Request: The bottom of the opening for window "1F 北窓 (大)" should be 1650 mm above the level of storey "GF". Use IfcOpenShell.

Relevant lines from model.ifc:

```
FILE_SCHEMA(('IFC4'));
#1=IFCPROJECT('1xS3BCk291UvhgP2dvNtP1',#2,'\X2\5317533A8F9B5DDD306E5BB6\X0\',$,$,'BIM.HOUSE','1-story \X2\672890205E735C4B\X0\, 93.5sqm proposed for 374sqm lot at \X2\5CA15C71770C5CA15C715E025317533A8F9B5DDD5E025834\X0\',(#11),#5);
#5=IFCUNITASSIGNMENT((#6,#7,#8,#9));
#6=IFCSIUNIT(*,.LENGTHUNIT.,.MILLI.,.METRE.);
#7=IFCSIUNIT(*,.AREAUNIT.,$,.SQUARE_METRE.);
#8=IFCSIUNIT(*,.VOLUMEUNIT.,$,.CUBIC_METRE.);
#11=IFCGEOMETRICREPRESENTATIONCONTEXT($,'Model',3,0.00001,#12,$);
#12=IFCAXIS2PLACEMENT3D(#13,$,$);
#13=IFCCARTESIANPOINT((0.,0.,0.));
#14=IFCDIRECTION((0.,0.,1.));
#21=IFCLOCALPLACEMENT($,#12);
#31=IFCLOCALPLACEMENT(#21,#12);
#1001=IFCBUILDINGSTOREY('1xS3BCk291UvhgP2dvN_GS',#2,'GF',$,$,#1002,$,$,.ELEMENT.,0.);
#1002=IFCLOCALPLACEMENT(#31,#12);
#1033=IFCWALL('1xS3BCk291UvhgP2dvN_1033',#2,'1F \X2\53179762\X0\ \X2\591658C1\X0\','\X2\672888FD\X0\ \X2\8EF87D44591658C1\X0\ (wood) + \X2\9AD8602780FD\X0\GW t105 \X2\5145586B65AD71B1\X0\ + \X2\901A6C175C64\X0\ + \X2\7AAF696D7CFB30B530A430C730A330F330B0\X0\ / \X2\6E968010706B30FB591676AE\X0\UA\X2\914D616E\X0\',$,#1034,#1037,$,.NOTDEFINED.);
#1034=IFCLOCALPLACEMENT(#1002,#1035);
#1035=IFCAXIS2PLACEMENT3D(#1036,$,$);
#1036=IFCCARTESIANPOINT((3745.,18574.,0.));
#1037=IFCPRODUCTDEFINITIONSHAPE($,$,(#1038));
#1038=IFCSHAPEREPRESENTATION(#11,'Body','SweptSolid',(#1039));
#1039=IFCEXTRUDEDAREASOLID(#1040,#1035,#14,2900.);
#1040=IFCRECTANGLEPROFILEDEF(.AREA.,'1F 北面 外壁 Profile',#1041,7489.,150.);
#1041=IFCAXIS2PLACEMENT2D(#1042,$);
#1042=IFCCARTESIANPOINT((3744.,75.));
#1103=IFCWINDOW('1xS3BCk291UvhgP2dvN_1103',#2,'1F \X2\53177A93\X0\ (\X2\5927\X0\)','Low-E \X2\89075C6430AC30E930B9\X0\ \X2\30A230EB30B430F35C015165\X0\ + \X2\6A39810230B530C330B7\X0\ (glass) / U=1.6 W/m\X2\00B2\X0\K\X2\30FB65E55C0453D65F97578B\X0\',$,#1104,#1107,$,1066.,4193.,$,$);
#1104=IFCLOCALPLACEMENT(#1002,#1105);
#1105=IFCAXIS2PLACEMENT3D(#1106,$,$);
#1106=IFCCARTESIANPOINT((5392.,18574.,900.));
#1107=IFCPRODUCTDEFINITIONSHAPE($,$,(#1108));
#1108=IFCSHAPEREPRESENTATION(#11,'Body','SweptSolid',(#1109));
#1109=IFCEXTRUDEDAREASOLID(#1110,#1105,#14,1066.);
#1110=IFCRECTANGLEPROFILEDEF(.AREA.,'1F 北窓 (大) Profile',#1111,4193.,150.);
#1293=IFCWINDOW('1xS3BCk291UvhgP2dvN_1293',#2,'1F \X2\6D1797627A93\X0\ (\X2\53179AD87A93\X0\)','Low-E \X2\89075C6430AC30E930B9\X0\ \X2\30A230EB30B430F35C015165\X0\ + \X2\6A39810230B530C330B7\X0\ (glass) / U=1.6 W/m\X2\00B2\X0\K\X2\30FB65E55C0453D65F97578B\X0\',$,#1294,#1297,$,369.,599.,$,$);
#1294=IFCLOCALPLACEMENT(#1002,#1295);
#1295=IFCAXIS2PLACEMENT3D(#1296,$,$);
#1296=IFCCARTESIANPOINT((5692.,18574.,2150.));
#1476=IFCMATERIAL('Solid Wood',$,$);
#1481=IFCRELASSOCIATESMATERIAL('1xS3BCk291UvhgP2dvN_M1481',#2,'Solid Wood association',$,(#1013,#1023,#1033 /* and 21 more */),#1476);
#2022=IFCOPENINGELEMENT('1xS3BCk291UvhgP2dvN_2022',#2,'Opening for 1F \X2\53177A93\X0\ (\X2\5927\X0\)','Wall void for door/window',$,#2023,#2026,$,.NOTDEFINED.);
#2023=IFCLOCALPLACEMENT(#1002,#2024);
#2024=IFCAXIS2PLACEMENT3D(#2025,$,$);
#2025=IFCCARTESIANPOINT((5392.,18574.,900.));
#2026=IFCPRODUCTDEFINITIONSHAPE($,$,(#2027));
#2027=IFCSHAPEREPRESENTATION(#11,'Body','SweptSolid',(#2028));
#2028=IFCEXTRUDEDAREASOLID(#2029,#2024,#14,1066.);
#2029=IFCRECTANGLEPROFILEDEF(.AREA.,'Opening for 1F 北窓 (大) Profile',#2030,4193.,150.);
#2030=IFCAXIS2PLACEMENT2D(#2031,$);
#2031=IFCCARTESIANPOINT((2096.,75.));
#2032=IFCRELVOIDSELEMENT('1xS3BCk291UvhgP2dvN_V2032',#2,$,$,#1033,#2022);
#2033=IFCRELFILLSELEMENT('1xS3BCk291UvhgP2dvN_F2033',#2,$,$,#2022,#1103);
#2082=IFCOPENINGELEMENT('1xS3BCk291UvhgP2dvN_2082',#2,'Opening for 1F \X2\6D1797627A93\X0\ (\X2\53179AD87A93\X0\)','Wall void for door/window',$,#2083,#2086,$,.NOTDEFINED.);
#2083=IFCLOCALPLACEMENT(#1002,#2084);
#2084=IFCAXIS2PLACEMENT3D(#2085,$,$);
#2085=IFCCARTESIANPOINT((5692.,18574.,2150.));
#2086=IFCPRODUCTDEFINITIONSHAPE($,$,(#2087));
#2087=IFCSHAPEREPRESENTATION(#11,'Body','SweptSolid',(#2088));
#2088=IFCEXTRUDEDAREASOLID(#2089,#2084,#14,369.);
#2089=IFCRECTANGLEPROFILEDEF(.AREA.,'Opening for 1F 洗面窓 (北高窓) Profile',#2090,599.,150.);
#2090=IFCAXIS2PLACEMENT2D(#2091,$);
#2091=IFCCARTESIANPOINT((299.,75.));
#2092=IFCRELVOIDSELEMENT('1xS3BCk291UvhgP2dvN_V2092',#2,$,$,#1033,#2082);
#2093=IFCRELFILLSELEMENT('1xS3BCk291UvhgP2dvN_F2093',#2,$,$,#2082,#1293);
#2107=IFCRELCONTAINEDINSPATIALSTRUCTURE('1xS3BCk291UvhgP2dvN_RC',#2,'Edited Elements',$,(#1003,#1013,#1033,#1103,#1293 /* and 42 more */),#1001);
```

```python
import numpy as np
import ifcopenshell
import ifcopenshell.api.geometry
import ifcopenshell.geom
import ifcopenshell.util.element
import ifcopenshell.util.placement
import ifcopenshell.util.shape
import ifcopenshell.util.unit

model = ifcopenshell.open("model.ifc")
unit_scale = ifcopenshell.util.unit.calculate_unit_scale(model)

window = model.by_guid("1xS3BCk291UvhgP2dvN_1103")
opening = window.FillsVoids[0].RelatingOpeningElement
storey = ifcopenshell.util.element.get_container(window, ifc_class="IfcBuildingStorey")
level = ifcopenshell.util.placement.get_local_placement(storey.ObjectPlacement)[2, 3]

# The opening's origin need not be at the sill, so measure its lowest point.
shape = ifcopenshell.geom.create_shape(ifcopenshell.geom.settings(), opening)
bottom = ifcopenshell.util.shape.get_shape_bottom_elevation(shape, shape.geometry) / unit_scale
dz = level + 1.65 / unit_scale - bottom

shift = np.array([0.0, 0.0, dz])
# The window is not placed relative to its opening, so move both.
for product in (opening, window):
    matrix = ifcopenshell.util.placement.get_local_placement(product.ObjectPlacement)
    matrix[:3, 3] += shift
    ifcopenshell.api.geometry.edit_object_placement(model, product=product, matrix=matrix, is_si=False)

print(f"moved by {dz * unit_scale:+.3f} m")

model.write("model-out.ifc")
```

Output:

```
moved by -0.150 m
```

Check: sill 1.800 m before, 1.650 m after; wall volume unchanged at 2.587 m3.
